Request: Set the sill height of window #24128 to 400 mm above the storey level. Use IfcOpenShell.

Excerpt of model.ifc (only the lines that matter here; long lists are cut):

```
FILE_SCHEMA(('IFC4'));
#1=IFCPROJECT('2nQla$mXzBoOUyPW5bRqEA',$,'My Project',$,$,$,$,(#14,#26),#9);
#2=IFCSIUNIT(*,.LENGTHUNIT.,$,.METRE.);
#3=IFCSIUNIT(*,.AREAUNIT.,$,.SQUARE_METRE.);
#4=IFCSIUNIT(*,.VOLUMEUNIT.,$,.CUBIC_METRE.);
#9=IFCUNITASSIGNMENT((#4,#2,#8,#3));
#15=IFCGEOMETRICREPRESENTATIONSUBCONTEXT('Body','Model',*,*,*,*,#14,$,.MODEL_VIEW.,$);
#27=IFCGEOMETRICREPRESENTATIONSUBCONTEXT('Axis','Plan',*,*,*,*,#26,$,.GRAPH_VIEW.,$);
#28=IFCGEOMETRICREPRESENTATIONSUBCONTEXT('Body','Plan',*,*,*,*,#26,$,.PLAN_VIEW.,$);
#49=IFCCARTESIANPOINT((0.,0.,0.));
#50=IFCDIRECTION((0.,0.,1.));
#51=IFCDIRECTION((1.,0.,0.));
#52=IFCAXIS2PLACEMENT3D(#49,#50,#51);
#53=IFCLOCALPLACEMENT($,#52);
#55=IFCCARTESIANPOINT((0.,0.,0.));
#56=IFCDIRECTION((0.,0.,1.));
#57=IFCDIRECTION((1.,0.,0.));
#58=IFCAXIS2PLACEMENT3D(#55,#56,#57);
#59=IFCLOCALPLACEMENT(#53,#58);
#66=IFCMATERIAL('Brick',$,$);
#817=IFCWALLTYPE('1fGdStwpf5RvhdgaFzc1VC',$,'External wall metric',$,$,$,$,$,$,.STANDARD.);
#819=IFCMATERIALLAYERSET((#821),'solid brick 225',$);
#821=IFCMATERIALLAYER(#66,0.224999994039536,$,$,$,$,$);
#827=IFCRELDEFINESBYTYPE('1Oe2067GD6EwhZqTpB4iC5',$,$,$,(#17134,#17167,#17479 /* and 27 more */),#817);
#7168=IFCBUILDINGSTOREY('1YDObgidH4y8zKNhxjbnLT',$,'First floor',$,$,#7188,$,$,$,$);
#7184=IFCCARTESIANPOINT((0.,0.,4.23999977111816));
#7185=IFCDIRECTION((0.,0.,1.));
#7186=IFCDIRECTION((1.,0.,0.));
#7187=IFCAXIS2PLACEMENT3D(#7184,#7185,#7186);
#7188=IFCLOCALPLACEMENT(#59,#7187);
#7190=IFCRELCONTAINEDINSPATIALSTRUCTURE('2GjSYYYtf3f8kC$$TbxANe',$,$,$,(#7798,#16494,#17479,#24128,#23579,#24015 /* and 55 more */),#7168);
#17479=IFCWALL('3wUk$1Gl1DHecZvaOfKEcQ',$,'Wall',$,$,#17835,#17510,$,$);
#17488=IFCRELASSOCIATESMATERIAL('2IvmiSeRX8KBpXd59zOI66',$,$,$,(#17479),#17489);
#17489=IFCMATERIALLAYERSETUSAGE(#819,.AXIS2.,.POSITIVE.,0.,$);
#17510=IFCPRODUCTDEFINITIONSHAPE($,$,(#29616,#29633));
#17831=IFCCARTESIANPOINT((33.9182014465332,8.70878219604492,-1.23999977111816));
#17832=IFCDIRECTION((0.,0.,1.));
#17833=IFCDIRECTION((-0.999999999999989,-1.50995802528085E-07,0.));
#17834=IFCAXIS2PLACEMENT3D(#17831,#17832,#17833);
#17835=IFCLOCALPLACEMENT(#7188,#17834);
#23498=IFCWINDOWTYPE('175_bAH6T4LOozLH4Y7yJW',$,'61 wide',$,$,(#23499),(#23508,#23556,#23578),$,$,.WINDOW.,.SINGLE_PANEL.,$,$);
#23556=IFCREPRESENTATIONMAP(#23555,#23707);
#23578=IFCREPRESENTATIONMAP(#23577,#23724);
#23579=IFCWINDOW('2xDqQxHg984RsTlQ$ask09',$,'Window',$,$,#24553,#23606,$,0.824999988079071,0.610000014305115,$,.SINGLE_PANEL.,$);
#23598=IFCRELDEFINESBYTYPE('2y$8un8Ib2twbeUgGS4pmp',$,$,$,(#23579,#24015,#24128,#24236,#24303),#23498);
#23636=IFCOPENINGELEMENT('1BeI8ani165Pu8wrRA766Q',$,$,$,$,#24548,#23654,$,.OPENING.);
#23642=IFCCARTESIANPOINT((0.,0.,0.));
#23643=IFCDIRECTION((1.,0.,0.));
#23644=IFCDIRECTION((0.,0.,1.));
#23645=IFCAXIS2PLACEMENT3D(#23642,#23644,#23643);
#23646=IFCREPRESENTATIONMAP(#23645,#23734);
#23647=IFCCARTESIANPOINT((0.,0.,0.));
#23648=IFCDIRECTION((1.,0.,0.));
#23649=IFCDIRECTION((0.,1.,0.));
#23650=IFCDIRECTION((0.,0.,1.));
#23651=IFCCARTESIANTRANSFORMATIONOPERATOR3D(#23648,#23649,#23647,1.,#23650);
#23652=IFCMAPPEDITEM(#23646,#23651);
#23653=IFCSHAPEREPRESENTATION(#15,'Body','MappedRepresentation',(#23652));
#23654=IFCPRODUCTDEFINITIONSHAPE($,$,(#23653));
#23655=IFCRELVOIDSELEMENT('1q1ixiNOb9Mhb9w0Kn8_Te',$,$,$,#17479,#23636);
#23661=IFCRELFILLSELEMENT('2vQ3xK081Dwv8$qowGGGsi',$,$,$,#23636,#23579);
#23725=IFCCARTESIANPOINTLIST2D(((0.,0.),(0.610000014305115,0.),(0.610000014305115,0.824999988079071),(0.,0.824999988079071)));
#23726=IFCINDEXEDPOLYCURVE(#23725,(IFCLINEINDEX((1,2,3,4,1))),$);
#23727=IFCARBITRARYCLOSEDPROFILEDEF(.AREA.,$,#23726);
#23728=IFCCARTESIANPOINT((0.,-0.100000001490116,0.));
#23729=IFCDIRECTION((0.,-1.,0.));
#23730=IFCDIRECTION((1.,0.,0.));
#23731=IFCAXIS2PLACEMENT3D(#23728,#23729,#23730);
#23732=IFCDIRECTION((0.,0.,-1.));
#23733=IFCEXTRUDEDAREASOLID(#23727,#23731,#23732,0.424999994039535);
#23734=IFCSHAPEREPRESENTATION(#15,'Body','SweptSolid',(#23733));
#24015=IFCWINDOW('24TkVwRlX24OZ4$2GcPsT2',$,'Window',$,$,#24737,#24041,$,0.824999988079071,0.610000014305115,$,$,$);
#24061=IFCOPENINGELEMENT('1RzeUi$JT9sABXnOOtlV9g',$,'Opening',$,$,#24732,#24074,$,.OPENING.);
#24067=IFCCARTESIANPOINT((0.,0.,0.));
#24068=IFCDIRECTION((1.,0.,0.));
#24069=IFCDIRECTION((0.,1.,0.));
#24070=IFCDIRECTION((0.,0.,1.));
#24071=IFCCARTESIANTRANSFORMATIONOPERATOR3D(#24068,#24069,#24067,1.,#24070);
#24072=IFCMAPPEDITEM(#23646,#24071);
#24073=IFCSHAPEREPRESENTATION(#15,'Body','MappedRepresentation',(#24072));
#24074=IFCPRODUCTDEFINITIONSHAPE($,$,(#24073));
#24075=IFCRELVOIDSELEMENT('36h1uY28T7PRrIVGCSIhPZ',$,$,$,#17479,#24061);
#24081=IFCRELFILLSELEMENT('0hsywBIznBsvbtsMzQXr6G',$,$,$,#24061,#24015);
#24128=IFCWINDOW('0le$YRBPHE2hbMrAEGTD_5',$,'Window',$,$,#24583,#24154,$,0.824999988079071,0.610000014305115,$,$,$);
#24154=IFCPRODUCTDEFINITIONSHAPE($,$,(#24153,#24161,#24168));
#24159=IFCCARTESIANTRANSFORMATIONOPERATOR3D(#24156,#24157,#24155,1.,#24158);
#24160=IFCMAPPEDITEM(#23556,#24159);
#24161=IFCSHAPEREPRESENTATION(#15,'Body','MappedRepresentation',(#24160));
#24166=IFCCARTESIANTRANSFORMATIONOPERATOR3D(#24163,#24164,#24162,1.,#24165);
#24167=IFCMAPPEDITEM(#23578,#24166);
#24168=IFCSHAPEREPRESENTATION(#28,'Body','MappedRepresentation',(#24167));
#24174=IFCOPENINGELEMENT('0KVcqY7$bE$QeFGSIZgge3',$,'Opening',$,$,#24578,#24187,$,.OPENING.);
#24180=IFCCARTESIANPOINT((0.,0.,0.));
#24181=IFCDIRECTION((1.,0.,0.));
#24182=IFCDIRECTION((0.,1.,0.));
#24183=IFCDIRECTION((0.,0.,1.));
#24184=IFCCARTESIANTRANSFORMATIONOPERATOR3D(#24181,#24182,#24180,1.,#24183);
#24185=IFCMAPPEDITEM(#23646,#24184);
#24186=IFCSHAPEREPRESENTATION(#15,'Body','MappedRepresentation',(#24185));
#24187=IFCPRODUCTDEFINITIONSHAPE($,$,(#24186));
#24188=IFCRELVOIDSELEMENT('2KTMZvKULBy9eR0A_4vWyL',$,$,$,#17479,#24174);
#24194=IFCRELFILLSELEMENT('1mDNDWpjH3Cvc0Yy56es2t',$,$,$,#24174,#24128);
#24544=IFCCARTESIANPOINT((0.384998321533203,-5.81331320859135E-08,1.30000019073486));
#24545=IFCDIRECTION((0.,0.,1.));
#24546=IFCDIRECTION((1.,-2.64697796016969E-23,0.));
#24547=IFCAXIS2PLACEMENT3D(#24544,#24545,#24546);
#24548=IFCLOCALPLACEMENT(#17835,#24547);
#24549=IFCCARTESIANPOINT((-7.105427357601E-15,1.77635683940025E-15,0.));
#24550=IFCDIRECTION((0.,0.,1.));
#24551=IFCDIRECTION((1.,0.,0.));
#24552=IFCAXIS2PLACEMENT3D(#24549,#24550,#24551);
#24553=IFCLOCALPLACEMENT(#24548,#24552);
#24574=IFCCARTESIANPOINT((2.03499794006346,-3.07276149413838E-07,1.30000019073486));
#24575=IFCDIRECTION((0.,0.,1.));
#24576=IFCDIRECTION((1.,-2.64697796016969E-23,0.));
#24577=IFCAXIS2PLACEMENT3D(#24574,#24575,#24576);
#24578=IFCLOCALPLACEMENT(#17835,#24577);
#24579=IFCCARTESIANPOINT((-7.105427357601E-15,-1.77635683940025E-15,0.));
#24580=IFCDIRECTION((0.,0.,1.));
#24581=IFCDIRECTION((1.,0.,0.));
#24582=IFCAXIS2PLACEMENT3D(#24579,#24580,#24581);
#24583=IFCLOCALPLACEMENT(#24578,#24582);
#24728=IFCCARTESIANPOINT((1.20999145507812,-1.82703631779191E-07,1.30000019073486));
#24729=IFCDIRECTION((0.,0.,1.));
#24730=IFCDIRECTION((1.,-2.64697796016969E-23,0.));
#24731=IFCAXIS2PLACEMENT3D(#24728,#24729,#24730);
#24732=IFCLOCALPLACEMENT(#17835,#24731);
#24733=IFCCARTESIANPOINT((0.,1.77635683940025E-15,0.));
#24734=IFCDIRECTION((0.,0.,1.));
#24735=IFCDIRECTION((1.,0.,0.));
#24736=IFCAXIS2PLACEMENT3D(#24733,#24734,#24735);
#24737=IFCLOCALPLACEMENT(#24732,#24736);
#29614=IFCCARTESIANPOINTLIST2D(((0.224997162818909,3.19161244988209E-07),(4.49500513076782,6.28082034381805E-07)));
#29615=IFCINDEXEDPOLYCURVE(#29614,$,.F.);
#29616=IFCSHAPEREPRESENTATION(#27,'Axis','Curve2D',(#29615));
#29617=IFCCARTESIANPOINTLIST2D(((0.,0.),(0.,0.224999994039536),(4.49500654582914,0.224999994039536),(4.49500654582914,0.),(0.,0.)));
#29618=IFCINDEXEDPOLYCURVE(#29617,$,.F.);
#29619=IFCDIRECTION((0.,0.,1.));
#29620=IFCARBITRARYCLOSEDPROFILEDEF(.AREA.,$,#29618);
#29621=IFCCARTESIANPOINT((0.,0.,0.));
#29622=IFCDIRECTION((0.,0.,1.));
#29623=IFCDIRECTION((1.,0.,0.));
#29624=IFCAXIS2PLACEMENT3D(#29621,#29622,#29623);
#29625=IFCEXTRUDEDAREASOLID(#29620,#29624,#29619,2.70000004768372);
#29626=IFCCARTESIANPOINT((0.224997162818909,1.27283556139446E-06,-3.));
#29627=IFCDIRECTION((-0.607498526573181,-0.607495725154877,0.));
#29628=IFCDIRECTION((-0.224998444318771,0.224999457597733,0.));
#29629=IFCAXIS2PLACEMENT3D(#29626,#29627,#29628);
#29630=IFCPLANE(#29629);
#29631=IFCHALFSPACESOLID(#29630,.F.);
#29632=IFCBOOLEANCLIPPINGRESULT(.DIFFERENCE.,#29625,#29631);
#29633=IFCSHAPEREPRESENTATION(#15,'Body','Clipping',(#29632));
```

```python
import numpy as np
import ifcopenshell
import ifcopenshell.api.geometry
import ifcopenshell.geom
import ifcopenshell.util.element
import ifcopenshell.util.placement
import ifcopenshell.util.shape
import ifcopenshell.util.unit

model = ifcopenshell.open("model.ifc")
unit_scale = ifcopenshell.util.unit.calculate_unit_scale(model)

window = model.by_guid("0le$YRBPHE2hbMrAEGTD_5")
opening = window.FillsVoids[0].RelatingOpeningElement
storey = ifcopenshell.util.element.get_container(window, ifc_class="IfcBuildingStorey")
level = ifcopenshell.util.placement.get_local_placement(storey.ObjectPlacement)[2, 3]

# The opening's origin need not be at the sill, so measure its lowest point.
shape = ifcopenshell.geom.create_shape(ifcopenshell.geom.settings(), opening)
bottom = ifcopenshell.util.shape.get_shape_bottom_elevation(shape, shape.geometry) / unit_scale
dz = level + 0.4 - bottom

shift = np.array([0.0, 0.0, dz])
# The window is placed relative to its opening, so it follows when the opening moves.
matrix = ifcopenshell.util.placement.get_local_placement(opening.ObjectPlacement)
matrix[:3, 3] += shift
ifcopenshell.api.geometry.edit_object_placement(
    model, product=opening, matrix=matrix, is_si=False, should_transform_children=True
)

print(f"moved by {dz * unit_scale:+.3f} m")

model.write("model_edited.ifc")
```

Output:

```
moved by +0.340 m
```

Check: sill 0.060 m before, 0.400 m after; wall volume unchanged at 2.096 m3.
